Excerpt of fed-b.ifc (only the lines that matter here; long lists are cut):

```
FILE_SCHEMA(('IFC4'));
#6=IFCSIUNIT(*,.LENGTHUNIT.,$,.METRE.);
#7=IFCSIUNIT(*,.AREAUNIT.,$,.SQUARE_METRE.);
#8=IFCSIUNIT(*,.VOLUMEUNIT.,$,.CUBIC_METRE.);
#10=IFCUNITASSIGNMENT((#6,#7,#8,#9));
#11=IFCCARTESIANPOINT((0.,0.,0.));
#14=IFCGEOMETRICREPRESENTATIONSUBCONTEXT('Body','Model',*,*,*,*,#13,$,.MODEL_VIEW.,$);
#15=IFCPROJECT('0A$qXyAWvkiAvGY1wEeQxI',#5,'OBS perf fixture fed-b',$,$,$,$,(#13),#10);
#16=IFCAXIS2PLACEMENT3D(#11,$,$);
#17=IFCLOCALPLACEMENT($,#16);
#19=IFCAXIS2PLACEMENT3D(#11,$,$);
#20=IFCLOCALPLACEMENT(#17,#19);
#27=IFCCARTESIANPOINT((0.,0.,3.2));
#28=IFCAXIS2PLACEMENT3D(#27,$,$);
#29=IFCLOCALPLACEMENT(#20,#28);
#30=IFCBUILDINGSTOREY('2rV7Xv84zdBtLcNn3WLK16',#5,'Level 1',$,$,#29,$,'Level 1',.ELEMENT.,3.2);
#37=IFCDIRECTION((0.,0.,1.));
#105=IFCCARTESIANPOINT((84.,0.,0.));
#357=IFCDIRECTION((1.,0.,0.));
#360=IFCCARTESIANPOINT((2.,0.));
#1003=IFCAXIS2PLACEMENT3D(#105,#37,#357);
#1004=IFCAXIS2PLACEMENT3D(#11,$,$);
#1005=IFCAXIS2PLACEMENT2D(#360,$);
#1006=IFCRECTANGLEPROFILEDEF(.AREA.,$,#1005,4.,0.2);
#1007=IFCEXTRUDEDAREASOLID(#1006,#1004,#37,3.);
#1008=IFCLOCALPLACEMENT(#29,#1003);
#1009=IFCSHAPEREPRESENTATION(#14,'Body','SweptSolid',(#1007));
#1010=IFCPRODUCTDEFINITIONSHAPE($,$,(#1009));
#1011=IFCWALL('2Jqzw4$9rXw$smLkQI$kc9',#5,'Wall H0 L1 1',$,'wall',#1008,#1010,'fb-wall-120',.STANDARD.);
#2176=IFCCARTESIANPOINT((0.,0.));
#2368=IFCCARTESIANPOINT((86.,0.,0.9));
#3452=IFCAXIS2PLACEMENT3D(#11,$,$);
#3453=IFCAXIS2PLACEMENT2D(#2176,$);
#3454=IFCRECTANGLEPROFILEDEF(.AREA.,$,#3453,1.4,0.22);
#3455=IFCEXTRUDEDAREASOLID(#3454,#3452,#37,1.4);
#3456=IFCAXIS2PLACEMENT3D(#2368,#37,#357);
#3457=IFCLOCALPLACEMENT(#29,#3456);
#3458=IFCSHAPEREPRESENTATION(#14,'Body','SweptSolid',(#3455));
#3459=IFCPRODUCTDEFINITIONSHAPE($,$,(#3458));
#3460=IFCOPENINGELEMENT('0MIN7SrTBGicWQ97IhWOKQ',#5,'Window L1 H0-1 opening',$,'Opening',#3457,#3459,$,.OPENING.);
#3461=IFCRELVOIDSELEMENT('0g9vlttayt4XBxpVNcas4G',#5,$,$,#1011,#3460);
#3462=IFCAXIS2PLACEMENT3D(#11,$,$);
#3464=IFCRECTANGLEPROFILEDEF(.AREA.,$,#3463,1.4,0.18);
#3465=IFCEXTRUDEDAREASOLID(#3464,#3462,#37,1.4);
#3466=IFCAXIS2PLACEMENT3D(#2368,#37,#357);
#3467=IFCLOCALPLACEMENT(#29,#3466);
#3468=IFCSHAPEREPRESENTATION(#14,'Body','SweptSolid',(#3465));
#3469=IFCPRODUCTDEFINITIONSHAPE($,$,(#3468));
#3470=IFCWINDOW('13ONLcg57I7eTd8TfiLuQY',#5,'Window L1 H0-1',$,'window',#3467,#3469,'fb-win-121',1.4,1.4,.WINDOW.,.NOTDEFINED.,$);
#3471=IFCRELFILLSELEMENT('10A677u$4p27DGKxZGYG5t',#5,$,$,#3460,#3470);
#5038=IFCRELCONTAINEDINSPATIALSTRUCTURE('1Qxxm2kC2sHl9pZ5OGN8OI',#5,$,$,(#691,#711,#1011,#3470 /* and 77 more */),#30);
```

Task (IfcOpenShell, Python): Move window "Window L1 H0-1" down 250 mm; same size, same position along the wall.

```python
import numpy as np
import ifcopenshell
import ifcopenshell.api.geometry
import ifcopenshell.util.placement
import ifcopenshell.util.unit

model = ifcopenshell.open("fed-b.ifc")
unit_scale = ifcopenshell.util.unit.calculate_unit_scale(model)

window = model.by_id(3470)
opening = window.FillsVoids[0].RelatingOpeningElement
dz = -0.25 / unit_scale

shift = np.array([0.0, 0.0, dz])
# The window is not placed relative to its opening, so move both.
for product in (opening, window):
    matrix = ifcopenshell.util.placement.get_local_placement(product.ObjectPlacement)
    matrix[:3, 3] += shift
    ifcopenshell.api.geometry.edit_object_placement(model, product=product, matrix=matrix, is_si=False)

print(f"moved by {dz * unit_scale:+.3f} m")

model.write("fed-b_v2.ifc")
```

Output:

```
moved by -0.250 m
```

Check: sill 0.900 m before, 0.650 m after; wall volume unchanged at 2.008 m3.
